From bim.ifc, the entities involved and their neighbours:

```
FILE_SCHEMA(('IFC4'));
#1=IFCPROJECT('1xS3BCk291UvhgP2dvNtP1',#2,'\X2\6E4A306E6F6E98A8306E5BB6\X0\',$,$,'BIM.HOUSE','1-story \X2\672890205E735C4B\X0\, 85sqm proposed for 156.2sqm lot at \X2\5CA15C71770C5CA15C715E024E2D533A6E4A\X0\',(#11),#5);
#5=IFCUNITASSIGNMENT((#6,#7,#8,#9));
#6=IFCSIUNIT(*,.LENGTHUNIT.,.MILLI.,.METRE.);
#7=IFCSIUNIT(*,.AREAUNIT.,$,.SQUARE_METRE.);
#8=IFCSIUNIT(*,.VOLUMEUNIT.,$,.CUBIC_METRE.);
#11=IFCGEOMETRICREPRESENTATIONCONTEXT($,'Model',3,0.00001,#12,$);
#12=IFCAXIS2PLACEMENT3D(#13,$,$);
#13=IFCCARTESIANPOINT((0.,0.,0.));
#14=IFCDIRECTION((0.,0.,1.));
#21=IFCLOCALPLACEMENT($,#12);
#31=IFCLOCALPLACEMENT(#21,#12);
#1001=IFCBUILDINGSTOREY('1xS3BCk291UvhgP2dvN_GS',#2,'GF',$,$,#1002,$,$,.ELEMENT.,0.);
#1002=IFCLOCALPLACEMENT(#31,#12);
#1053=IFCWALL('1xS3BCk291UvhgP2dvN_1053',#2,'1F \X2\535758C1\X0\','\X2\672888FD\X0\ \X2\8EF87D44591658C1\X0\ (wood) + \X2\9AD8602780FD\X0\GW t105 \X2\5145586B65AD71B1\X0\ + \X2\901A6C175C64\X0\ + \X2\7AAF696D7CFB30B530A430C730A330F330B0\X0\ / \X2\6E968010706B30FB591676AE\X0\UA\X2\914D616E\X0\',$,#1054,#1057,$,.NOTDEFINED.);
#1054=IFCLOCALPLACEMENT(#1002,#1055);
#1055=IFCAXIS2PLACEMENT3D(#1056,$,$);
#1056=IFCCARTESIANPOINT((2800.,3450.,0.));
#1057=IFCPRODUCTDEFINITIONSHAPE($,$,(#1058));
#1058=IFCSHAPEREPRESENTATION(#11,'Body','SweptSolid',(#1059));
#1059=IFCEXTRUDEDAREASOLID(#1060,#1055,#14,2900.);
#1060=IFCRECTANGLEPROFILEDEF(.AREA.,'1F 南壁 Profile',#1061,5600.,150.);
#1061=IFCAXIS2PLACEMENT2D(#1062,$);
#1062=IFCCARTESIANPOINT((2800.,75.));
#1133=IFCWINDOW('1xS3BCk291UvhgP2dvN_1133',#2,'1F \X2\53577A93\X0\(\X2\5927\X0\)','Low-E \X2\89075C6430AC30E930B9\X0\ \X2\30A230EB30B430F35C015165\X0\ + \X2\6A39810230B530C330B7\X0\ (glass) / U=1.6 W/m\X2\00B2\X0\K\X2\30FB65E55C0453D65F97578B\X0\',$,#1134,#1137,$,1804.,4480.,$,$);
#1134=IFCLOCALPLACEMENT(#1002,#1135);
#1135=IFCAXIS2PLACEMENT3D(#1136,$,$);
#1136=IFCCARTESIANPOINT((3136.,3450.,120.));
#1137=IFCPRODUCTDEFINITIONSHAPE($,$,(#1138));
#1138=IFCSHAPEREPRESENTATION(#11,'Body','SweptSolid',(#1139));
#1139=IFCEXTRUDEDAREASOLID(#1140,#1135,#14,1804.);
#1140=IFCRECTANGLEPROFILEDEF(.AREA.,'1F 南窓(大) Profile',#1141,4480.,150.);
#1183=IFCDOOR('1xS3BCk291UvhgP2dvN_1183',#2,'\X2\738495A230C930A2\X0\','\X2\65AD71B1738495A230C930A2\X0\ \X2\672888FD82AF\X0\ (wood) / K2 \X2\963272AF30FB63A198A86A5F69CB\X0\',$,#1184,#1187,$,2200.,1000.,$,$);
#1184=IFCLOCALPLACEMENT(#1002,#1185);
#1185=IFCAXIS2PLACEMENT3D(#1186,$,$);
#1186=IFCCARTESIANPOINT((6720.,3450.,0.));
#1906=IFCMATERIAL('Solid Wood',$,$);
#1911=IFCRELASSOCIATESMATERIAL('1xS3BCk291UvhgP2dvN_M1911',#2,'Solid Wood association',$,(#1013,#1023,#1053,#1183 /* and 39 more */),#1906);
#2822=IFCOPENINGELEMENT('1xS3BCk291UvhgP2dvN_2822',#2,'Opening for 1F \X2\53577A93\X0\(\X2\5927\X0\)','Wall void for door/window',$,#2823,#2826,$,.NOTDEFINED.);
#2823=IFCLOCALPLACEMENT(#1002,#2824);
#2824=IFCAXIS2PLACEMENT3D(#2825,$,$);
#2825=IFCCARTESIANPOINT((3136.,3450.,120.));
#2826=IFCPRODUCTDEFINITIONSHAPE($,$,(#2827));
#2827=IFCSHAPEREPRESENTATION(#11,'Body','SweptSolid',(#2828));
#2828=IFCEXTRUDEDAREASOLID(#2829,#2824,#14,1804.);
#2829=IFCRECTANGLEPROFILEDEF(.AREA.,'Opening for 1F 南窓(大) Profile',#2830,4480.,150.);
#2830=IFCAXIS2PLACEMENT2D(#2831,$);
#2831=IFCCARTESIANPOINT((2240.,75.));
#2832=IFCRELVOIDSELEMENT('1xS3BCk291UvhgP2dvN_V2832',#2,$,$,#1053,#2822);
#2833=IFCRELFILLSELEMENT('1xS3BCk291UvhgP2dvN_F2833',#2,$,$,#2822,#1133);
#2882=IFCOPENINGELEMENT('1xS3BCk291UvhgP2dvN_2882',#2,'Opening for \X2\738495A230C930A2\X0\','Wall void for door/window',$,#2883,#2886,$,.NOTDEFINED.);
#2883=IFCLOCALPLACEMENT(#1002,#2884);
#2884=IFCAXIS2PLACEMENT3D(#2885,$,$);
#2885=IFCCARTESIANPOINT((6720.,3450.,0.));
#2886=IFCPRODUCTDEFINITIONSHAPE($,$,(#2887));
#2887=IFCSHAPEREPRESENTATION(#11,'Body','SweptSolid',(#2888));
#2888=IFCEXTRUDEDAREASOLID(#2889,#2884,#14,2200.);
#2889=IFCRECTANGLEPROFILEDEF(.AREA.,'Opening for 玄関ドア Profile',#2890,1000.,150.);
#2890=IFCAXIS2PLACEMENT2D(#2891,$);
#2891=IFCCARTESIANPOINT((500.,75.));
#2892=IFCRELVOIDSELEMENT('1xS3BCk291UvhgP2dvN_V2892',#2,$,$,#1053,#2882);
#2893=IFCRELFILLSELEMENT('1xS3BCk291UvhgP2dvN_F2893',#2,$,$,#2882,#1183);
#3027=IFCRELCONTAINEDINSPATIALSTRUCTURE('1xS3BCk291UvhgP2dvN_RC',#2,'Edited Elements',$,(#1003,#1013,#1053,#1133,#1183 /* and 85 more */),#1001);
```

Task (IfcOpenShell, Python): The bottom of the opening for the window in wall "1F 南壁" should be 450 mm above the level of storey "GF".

```python
import numpy as np
import ifcopenshell
import ifcopenshell.api.geometry
import ifcopenshell.geom
import ifcopenshell.util.element
import ifcopenshell.util.placement
import ifcopenshell.util.shape
import ifcopenshell.util.unit

model = ifcopenshell.open("bim.ifc")
unit_scale = ifcopenshell.util.unit.calculate_unit_scale(model)

window = model.by_guid("1xS3BCk291UvhgP2dvN_1133")
opening = window.FillsVoids[0].RelatingOpeningElement
storey = ifcopenshell.util.element.get_container(window, ifc_class="IfcBuildingStorey")
level = ifcopenshell.util.placement.get_local_placement(storey.ObjectPlacement)[2, 3]

# The opening's origin need not be at the sill, so measure its lowest point.
shape = ifcopenshell.geom.create_shape(ifcopenshell.geom.settings(), opening)
bottom = ifcopenshell.util.shape.get_shape_bottom_elevation(shape, shape.geometry) / unit_scale
dz = level + 0.45 / unit_scale - bottom

shift = np.array([0.0, 0.0, dz])
# The window is not placed relative to its opening, so move both.
for product in (opening, window):
    matrix = ifcopenshell.util.placement.get_local_placement(product.ObjectPlacement)
    matrix[:3, 3] += shift
    ifcopenshell.api.geometry.edit_object_placement(model, product=product, matrix=matrix, is_si=False)

print(f"moved by {dz * unit_scale:+.3f} m")

model.write("bim_updated.ifc")
```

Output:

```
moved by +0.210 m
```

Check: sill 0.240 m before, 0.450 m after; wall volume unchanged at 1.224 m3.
